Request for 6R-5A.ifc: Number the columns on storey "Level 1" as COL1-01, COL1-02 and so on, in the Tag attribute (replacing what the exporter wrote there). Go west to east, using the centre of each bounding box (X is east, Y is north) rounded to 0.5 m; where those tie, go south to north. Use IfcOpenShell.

First a look at what the model holds.

```python
import ifcopenshell
import ifcopenshell.util.element
import ifcopenshell.util.placement

model = ifcopenshell.open("6R-5A.ifc")
print(model.schema)
storey = next(s for s in model.by_type("IfcBuildingStorey") if s.Name == "Level 1")
columns = [e for e in ifcopenshell.util.element.get_decomposition(storey) if e.is_a("IfcColumn")]
for e in sorted(columns, key=lambda e: e.id()):
    origin = ifcopenshell.util.placement.get_local_placement(e.ObjectPlacement)[:3, 3]
    print(e.id(), e.Tag, e.Name, origin.round(2) + 0.0, sep=" | ")
```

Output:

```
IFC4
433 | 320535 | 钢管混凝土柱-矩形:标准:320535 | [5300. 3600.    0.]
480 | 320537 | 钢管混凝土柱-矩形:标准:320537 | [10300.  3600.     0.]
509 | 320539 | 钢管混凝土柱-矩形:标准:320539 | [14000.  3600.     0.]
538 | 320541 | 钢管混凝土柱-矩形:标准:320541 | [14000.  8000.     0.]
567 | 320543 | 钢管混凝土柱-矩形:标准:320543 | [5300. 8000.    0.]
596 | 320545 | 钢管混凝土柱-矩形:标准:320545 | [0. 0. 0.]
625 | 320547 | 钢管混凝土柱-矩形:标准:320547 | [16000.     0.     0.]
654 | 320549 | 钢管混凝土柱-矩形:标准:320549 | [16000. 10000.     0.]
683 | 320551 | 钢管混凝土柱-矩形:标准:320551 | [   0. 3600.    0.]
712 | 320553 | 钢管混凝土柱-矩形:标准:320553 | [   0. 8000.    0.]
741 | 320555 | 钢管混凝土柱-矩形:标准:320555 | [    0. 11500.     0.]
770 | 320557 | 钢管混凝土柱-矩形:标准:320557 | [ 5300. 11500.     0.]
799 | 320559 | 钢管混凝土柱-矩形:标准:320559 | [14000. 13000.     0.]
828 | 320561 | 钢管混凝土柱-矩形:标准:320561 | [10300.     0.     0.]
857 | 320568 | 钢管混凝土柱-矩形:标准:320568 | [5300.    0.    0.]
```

```python
import ifcopenshell
import ifcopenshell.geom
import ifcopenshell.util.element
import ifcopenshell.util.shape

model = ifcopenshell.open("6R-5A.ifc")
settings = ifcopenshell.geom.settings()
settings.set("use-world-coords", True)


def centre(element):
    shape = ifcopenshell.geom.create_shape(settings, element)
    return ifcopenshell.util.shape.get_bbox_centroid(shape.geometry)


storey = next(s for s in model.by_type("IfcBuildingStorey") if s.Name == "Level 1")
columns = [e for e in ifcopenshell.util.element.get_decomposition(storey) if e.is_a("IfcColumn")]

# Insertion points can sit at a corner or the storey origin, so sort by the geometry (in metres).
centres = {e: centre(e) for e in columns}
columns.sort(key=lambda e: (round(centres[e][0] / 0.5), centres[e][1]))

for i, e in enumerate(columns, start=1):
    number = f"COL1-{i:02d}"
    e.Tag = number
    print(e.id(), number)

model.write("6R-5A_updated.ifc")
```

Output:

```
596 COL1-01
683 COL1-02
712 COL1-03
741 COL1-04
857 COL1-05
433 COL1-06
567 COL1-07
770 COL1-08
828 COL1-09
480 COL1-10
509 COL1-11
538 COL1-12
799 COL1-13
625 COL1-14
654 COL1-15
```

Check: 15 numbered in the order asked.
